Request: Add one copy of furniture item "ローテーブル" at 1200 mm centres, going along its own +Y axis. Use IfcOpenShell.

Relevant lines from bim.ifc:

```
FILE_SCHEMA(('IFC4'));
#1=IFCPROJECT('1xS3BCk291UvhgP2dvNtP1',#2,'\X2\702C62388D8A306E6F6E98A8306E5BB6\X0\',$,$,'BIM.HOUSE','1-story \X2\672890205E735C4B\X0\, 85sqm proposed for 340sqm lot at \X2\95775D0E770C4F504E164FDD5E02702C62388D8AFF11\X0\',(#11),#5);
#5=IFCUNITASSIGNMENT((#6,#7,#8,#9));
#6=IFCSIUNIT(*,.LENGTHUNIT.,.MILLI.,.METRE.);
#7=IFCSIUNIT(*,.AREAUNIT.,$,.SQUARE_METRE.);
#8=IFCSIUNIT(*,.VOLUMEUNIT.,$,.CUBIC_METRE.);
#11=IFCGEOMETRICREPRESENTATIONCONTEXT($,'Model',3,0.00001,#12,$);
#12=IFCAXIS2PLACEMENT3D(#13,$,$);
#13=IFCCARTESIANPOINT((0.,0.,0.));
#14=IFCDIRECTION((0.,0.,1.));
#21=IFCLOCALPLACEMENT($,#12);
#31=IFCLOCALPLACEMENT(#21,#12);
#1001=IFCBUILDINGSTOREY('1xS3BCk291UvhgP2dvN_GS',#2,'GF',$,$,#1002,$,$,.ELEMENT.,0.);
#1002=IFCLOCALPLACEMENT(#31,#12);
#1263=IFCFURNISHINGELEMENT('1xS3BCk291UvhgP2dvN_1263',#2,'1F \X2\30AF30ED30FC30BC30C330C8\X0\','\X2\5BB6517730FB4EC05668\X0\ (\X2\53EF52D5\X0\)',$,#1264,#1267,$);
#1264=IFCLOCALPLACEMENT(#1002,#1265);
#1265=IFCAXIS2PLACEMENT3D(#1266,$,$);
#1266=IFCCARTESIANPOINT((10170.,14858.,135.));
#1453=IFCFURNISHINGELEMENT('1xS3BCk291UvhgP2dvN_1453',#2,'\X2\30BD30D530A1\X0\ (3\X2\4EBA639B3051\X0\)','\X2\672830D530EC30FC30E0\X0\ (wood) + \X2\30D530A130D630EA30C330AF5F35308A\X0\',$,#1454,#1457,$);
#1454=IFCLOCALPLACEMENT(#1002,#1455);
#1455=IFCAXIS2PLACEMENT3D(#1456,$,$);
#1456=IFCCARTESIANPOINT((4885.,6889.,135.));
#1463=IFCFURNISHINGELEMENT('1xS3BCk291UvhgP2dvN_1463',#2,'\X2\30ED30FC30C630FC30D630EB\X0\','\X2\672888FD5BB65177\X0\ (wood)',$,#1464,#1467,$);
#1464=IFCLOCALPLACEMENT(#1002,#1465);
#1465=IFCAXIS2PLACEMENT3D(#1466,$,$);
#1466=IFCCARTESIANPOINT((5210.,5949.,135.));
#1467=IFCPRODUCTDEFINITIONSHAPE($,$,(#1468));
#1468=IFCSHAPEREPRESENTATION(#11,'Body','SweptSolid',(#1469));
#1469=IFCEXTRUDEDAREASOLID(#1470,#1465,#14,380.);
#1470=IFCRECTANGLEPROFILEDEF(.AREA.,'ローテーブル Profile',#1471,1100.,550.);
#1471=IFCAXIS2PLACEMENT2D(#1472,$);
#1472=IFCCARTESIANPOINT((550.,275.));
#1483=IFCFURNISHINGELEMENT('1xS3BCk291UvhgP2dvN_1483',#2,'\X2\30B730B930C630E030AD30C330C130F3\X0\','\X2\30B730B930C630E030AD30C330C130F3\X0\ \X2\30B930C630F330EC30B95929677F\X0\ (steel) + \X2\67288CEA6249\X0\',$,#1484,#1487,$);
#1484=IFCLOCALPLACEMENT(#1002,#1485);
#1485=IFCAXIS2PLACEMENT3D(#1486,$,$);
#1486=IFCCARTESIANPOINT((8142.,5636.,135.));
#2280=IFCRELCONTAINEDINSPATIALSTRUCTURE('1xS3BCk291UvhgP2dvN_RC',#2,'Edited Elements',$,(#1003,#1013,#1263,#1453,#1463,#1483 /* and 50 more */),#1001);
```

```python
import ifcopenshell
import ifcopenshell.api.geometry
import ifcopenshell.api.root
import ifcopenshell.util.element
import ifcopenshell.util.placement
import ifcopenshell.util.unit

model = ifcopenshell.open("bim.ifc")
unit_scale = ifcopenshell.util.unit.calculate_unit_scale(model)


def reuse_history(source, copy):
    """copy_class also copies each property set's owner history, people and application; keep the originals."""
    for rel in copy.IsDefinedBy:
        if rel.is_a("IfcRelDefinesByProperties") and (history := rel.RelatingPropertyDefinition.OwnerHistory):
            rel.RelatingPropertyDefinition.OwnerHistory = source.OwnerHistory
            ifcopenshell.util.element.remove_deep2(model, history)


source = model.by_guid("1xS3BCk291UvhgP2dvN_1463")
base = ifcopenshell.util.placement.get_local_placement(source.ObjectPlacement)
step = base[:3, 1] * 1.2 / unit_scale

for i in range(1, 2):
    copy = ifcopenshell.api.root.copy_class(model, product=source)
    copy.Representation = ifcopenshell.util.element.copy_deep(
        model, source.Representation, exclude=["IfcGeometricRepresentationContext", "IfcRepresentationMap"]
    )
    reuse_history(source, copy)
    matrix = base.copy()
    matrix[:3, 3] += i * step
    print("added at", matrix[:3, 3].round(3) + 0.0)
    ifcopenshell.api.geometry.edit_object_placement(model, product=copy, matrix=matrix, is_si=False)

model.write("bim_edited.ifc")
```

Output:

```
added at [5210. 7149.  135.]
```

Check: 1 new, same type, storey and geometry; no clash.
